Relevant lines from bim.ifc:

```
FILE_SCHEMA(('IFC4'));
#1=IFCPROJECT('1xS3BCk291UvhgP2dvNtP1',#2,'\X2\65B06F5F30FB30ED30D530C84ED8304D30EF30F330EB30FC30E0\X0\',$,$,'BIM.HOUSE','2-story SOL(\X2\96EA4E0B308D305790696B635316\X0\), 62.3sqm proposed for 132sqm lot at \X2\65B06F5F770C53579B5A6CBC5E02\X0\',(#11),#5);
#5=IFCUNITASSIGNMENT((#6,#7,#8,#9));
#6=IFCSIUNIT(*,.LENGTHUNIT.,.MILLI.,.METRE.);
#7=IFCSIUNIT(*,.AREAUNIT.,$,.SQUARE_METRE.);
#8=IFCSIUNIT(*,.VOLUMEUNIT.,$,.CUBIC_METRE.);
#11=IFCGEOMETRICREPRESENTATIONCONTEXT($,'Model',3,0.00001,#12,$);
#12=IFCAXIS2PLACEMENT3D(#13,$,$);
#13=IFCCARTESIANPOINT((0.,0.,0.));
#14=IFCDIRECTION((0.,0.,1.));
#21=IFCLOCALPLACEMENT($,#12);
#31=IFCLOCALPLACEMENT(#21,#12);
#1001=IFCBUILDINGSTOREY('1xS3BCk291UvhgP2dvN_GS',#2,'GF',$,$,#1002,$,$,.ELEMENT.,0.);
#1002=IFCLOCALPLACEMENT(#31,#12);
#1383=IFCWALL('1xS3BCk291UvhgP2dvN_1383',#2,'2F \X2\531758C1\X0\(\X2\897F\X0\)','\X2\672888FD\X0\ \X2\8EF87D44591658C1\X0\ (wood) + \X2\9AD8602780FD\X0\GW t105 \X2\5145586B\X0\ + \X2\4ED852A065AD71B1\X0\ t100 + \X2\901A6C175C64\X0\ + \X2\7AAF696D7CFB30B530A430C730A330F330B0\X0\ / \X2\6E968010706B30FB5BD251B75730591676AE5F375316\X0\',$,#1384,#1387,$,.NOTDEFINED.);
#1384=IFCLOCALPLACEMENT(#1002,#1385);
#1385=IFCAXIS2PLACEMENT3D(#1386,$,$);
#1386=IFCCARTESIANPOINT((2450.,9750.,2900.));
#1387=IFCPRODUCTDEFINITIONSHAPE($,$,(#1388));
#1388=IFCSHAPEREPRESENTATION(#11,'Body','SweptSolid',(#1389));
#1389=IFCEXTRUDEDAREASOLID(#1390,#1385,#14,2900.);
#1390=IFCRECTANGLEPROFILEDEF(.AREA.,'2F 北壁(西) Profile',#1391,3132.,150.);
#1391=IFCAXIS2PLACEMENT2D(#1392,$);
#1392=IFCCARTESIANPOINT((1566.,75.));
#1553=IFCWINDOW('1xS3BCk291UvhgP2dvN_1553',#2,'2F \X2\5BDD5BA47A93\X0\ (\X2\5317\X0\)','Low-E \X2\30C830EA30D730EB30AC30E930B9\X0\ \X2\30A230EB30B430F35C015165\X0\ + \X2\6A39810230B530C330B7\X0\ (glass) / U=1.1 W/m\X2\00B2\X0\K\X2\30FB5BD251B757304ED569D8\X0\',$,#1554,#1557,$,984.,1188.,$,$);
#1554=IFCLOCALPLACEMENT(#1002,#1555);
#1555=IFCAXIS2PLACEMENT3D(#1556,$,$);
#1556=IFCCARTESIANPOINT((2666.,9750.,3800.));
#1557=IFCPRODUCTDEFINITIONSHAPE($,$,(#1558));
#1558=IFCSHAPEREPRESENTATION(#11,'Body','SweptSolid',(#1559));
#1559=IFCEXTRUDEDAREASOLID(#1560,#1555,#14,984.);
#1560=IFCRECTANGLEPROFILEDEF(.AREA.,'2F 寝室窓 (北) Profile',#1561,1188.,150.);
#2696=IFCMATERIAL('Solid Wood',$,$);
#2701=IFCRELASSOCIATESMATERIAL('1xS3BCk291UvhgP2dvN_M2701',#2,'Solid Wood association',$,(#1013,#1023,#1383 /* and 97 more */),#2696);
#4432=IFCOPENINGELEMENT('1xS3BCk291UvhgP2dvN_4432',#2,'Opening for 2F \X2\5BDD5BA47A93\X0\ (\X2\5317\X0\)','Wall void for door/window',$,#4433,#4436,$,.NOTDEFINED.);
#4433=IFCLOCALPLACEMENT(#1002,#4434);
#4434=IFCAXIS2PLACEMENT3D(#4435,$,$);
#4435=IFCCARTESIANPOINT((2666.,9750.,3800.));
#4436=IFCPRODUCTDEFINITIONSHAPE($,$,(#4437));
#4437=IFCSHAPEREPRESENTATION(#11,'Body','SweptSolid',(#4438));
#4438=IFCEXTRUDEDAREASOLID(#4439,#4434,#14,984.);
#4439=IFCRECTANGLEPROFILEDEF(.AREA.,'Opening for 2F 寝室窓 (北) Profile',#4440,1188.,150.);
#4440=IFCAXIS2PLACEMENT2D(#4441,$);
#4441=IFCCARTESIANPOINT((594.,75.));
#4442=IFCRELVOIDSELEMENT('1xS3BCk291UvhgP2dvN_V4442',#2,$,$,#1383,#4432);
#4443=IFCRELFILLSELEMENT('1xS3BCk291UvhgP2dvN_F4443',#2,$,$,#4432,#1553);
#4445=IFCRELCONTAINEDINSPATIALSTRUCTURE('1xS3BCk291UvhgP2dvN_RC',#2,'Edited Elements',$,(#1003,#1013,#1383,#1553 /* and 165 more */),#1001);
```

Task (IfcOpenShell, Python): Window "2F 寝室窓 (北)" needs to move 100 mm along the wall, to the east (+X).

```python
import ifcopenshell
import ifcopenshell.api.geometry
import ifcopenshell.util.placement

model = ifcopenshell.open("bim.ifc")

window = model.by_id(1553)
opening = window.FillsVoids[0].RelatingOpeningElement
wall = opening.VoidsElements[0].RelatingBuildingElement

wall_matrix = ifcopenshell.util.placement.get_local_placement(wall.ObjectPlacement)
shift = wall_matrix[:3, 0] * 100.0
before = ifcopenshell.util.placement.get_local_placement(window.ObjectPlacement)[:3, 3].copy()

# The window is not placed relative to its opening, so move both.
for product in (opening, window):
    matrix = ifcopenshell.util.placement.get_local_placement(product.ObjectPlacement)
    matrix[:3, 3] += shift
    ifcopenshell.api.geometry.edit_object_placement(model, product=product, matrix=matrix, is_si=False)

after = ifcopenshell.util.placement.get_local_placement(window.ObjectPlacement)[:3, 3]
print("window moved by", (after - before).round(3) + 0.0)

model.write("bim_rev.ifc")
```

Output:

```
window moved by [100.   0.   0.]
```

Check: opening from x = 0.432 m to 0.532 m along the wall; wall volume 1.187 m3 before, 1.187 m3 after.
